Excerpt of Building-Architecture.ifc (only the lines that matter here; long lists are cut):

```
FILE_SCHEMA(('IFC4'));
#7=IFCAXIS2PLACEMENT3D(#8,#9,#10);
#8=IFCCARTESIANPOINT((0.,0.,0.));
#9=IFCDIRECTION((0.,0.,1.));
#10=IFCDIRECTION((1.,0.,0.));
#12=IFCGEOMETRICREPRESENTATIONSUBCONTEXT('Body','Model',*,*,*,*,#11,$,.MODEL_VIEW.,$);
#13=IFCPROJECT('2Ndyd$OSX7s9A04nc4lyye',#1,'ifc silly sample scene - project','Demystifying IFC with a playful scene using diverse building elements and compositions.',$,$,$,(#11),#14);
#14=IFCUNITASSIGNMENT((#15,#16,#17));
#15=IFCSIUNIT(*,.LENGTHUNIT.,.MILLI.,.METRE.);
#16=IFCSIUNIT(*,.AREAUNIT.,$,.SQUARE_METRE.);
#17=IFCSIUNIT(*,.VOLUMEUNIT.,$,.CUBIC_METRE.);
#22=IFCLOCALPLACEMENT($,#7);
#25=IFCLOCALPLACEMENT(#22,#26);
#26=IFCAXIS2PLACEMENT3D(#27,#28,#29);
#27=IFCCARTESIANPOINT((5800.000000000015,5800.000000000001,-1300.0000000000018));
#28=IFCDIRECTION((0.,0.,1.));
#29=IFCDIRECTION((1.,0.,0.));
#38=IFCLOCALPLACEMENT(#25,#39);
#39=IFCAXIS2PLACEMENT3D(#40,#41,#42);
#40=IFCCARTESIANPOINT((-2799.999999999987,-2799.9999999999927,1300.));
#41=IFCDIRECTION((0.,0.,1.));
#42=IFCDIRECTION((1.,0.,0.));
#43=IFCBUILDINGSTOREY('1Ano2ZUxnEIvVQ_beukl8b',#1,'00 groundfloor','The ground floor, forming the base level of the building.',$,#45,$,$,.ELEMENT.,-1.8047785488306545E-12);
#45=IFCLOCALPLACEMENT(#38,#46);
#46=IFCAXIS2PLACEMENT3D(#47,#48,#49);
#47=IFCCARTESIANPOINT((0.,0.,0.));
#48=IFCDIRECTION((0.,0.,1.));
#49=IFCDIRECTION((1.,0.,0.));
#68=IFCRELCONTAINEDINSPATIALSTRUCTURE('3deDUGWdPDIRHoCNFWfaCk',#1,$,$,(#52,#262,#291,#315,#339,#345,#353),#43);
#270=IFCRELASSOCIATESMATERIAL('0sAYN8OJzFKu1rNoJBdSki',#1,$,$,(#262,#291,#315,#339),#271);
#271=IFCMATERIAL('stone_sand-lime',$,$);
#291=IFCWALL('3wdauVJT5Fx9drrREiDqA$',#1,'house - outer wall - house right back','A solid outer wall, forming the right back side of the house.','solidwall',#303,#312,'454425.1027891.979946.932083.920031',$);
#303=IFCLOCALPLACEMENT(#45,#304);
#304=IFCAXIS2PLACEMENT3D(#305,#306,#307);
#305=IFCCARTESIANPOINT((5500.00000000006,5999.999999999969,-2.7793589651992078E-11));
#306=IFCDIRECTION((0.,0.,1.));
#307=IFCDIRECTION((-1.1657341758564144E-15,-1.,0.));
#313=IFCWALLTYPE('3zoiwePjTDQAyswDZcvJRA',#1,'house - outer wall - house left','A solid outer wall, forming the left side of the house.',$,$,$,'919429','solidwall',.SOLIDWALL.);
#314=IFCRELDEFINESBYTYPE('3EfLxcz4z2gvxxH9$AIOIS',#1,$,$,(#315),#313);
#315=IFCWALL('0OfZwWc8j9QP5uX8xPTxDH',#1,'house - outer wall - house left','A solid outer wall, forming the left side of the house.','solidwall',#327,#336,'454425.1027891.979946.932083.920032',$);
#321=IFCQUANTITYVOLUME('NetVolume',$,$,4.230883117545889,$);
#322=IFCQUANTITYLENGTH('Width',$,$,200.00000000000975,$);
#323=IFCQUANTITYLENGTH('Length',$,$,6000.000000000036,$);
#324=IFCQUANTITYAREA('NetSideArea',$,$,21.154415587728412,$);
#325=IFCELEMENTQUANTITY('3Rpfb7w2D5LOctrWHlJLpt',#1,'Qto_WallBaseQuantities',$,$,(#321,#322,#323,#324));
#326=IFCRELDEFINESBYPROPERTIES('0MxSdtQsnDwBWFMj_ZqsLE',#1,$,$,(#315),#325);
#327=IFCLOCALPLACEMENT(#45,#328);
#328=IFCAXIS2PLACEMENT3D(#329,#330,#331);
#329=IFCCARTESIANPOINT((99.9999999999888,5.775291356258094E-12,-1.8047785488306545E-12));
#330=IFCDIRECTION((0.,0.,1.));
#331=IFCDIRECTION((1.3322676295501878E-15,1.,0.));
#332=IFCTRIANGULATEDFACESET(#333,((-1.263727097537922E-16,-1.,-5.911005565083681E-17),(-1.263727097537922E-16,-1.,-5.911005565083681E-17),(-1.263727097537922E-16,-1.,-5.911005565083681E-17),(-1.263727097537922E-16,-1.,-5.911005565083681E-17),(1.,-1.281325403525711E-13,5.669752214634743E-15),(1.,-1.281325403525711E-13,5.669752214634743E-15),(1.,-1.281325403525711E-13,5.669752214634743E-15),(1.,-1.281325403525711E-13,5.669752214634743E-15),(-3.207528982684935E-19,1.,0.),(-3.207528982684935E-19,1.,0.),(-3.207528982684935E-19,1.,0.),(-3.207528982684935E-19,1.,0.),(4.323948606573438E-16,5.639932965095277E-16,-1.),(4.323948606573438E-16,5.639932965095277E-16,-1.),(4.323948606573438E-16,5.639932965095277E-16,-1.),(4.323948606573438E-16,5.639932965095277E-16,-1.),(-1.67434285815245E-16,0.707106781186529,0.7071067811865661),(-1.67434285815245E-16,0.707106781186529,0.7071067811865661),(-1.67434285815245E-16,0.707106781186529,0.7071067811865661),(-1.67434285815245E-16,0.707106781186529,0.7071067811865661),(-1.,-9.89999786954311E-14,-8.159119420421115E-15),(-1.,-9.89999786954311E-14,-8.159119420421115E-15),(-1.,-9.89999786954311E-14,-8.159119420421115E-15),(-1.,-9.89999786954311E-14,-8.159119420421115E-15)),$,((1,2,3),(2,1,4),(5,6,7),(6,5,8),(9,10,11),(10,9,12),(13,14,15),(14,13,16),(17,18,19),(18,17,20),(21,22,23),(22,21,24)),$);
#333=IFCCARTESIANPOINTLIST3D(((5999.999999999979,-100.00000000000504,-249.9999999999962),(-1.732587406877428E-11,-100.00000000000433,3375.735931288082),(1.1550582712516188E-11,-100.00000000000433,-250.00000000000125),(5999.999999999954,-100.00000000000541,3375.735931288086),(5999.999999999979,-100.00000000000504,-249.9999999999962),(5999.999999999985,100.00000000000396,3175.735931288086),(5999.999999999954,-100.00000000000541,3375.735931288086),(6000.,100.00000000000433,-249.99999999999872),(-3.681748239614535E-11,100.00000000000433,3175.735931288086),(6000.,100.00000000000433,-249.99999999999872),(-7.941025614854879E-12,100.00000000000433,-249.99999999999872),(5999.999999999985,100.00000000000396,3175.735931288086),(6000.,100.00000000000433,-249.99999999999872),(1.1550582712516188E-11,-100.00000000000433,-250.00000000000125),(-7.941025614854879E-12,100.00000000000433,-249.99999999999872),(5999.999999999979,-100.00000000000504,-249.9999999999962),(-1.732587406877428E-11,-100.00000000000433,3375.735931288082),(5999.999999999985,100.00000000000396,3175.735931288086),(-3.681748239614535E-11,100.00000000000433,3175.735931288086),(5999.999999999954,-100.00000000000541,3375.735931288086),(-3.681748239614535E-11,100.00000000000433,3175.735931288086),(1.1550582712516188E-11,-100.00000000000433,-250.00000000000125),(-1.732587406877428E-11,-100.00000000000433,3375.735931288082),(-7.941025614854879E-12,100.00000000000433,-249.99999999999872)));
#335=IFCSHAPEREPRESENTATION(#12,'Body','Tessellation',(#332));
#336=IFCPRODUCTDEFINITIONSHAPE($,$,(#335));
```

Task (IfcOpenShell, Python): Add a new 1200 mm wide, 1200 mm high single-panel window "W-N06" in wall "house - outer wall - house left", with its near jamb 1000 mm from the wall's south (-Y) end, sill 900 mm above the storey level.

```python
import numpy as np
import ifcopenshell
import ifcopenshell.api.feature
import ifcopenshell.api.geometry
import ifcopenshell.api.pset
import ifcopenshell.api.root
import ifcopenshell.api.spatial
import ifcopenshell.geom
import ifcopenshell.util.element
import ifcopenshell.util.placement
import ifcopenshell.util.representation
import ifcopenshell.util.shape
import ifcopenshell.util.unit

model = ifcopenshell.open("Building-Architecture.ifc")
unit_scale = ifcopenshell.util.unit.calculate_unit_scale(model)
area_scale = ifcopenshell.util.unit.calculate_unit_scale(model, "AREAUNIT")
volume_scale = ifcopenshell.util.unit.calculate_unit_scale(model, "VOLUMEUNIT")
settings = ifcopenshell.geom.settings()


def volume(element):
    """Net volume in cubic metres, openings subtracted."""
    shape = ifcopenshell.geom.create_shape(settings, element)
    return ifcopenshell.util.shape.get_volume(shape.geometry)


wall = model.by_guid("0OfZwWc8j9QP5uX8xPTxDH")
storey = ifcopenshell.util.element.get_container(wall, ifc_class="IfcBuildingStorey")
context = ifcopenshell.util.representation.get_context(model, "Model", "Body", "MODEL_VIEW")
before = volume(wall)

width, height, from_end, sill = 1.2, 1.2, 1, 0.9  # metres

# The wall runs along its own X axis, and the end named is its -X end.
wall_shape = ifcopenshell.geom.create_shape(settings, wall)
x, y, z = ifcopenshell.util.shape.get_vertices(wall_shape.geometry).T
start = x.min() + from_end
face, thickness = float(y.min()), float(y.max() - y.min())
wall_matrix = ifcopenshell.util.placement.get_local_placement(wall.ObjectPlacement)
level = ifcopenshell.util.placement.get_local_placement(storey.ObjectPlacement)[2, 3]


def in_wall(x, y):
    """Placement at x, y metres in the wall's axes, at sill height."""
    matrix = wall_matrix.copy()
    matrix[:, 3] = wall_matrix @ np.array([x / unit_scale, y / unit_scale, 0.0, 1.0])
    matrix[2, 3] = level + sill / unit_scale
    return matrix


# Opening: a box that overshoots both wall faces by 50 mm.
opening = ifcopenshell.api.root.create_entity(model, ifc_class="IfcOpeningElement", predefined_type="OPENING")
box = ifcopenshell.api.geometry.add_wall_representation(
    model, context=context, length=width, height=height, thickness=thickness + 0.1
)
ifcopenshell.api.geometry.assign_representation(model, product=opening, representation=box)
ifcopenshell.api.geometry.edit_object_placement(model, product=opening, matrix=in_wall(start, face - 0.05), is_si=False)
ifcopenshell.api.feature.add_feature(model, feature=opening, element=wall)

window = ifcopenshell.api.root.create_entity(model, ifc_class="IfcWindow", name="W-N06", predefined_type="WINDOW")
window.OverallWidth, window.OverallHeight = width / unit_scale, height / unit_scale
window.PartitioningType = "SINGLE_PANEL"
body = ifcopenshell.api.geometry.add_window_representation(
    model,
    context=context,
    overall_width=window.OverallWidth,
    overall_height=window.OverallHeight,
    partition_type="SINGLE_PANEL",
)
ifcopenshell.api.geometry.assign_representation(model, product=window, representation=body)
ifcopenshell.api.spatial.assign_container(model, products=[window], relating_structure=storey)
ifcopenshell.api.feature.add_filling(model, opening=opening, element=window)

# Centre the window in the wall's thickness.
ifcopenshell.api.geometry.edit_object_placement(model, product=window, matrix=in_wall(start, face), is_si=False)
window_shape = ifcopenshell.geom.create_shape(settings, window)
depth = ifcopenshell.util.shape.get_vertices(window_shape.geometry)[:, 1]
offset = face + thickness / 2 - (depth.min() + depth.max()) / 2
ifcopenshell.api.geometry.edit_object_placement(model, product=window, matrix=in_wall(start, offset), is_si=False)

after = volume(wall)

# Update the wall's stored quantities.
qto = model.by_id(ifcopenshell.util.element.get_pset(wall, "Qto_WallBaseQuantities", should_inherit=False)["id"])
ifcopenshell.api.pset.edit_qto(model, qto=qto, properties={
    "NetVolume": after / volume_scale,
    "NetSideArea": after / thickness / area_scale,
})

print(f"wall volume {before:.3f} -> {after:.3f} m3")

model.write("Building-Architecture_rev.ifc")
```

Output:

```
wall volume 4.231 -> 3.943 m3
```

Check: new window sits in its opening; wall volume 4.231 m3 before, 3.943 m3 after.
